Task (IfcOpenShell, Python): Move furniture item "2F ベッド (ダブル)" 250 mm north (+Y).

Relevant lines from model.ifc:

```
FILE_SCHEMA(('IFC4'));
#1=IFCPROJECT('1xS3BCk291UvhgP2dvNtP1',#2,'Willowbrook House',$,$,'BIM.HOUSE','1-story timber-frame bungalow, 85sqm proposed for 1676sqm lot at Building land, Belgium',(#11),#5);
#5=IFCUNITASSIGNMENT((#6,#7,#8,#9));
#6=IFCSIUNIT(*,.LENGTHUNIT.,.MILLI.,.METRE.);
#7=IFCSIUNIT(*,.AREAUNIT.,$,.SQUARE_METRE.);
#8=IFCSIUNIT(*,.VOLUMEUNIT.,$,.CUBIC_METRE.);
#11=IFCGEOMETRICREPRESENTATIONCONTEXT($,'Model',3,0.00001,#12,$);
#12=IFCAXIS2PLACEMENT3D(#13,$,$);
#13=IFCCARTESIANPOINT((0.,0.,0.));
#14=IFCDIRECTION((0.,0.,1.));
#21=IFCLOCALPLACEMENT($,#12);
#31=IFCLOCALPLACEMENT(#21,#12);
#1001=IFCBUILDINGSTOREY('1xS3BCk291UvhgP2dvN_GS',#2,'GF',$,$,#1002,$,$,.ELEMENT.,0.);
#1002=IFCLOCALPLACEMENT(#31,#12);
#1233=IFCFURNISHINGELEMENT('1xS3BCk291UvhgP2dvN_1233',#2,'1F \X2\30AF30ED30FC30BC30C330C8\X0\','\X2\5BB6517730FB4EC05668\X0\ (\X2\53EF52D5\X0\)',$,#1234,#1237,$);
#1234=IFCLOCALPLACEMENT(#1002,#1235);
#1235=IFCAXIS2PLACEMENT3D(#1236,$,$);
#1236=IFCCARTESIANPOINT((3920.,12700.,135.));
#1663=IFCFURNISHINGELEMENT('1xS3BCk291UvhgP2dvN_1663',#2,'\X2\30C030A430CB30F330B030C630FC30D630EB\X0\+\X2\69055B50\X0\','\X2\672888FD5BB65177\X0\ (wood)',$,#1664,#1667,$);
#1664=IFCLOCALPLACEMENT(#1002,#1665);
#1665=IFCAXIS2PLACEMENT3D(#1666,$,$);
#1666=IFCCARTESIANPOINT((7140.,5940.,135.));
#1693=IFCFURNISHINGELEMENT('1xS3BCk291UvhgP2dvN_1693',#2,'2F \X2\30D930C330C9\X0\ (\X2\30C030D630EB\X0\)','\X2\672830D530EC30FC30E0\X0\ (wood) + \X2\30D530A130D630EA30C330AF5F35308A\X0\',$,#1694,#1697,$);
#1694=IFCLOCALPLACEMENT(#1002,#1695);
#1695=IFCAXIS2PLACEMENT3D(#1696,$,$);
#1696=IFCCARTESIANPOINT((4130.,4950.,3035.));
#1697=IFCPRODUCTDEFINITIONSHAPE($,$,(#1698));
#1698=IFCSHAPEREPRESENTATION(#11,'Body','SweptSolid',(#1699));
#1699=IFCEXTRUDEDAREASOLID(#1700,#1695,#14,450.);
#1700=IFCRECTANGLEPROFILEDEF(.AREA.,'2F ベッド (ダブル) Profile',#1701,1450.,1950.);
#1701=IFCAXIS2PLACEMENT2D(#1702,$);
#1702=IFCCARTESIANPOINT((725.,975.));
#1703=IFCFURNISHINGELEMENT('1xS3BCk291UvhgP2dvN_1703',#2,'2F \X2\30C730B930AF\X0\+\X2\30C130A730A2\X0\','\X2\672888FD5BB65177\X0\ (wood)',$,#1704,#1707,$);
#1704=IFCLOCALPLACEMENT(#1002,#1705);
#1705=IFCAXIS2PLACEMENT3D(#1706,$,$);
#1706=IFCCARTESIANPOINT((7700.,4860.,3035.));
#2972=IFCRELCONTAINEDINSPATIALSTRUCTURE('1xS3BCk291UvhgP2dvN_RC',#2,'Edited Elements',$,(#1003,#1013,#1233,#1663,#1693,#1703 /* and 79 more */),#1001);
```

```python
import ifcopenshell
import ifcopenshell.api.geometry
import ifcopenshell.util.placement

model = ifcopenshell.open("model.ifc")

item = model.by_guid("1xS3BCk291UvhgP2dvN_1693")
matrix = ifcopenshell.util.placement.get_local_placement(item.ObjectPlacement)
matrix[1, 3] += 250.0
ifcopenshell.api.geometry.edit_object_placement(model, product=item, matrix=matrix, is_si=False)

print(ifcopenshell.util.placement.get_local_placement(item.ObjectPlacement).round(3) + 0.0)

model.write("model_v2.ifc")
```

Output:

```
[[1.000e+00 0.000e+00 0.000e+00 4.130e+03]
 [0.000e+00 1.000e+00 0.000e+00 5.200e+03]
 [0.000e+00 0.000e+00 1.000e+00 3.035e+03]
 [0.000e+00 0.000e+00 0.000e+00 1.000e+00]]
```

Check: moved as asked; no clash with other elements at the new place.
